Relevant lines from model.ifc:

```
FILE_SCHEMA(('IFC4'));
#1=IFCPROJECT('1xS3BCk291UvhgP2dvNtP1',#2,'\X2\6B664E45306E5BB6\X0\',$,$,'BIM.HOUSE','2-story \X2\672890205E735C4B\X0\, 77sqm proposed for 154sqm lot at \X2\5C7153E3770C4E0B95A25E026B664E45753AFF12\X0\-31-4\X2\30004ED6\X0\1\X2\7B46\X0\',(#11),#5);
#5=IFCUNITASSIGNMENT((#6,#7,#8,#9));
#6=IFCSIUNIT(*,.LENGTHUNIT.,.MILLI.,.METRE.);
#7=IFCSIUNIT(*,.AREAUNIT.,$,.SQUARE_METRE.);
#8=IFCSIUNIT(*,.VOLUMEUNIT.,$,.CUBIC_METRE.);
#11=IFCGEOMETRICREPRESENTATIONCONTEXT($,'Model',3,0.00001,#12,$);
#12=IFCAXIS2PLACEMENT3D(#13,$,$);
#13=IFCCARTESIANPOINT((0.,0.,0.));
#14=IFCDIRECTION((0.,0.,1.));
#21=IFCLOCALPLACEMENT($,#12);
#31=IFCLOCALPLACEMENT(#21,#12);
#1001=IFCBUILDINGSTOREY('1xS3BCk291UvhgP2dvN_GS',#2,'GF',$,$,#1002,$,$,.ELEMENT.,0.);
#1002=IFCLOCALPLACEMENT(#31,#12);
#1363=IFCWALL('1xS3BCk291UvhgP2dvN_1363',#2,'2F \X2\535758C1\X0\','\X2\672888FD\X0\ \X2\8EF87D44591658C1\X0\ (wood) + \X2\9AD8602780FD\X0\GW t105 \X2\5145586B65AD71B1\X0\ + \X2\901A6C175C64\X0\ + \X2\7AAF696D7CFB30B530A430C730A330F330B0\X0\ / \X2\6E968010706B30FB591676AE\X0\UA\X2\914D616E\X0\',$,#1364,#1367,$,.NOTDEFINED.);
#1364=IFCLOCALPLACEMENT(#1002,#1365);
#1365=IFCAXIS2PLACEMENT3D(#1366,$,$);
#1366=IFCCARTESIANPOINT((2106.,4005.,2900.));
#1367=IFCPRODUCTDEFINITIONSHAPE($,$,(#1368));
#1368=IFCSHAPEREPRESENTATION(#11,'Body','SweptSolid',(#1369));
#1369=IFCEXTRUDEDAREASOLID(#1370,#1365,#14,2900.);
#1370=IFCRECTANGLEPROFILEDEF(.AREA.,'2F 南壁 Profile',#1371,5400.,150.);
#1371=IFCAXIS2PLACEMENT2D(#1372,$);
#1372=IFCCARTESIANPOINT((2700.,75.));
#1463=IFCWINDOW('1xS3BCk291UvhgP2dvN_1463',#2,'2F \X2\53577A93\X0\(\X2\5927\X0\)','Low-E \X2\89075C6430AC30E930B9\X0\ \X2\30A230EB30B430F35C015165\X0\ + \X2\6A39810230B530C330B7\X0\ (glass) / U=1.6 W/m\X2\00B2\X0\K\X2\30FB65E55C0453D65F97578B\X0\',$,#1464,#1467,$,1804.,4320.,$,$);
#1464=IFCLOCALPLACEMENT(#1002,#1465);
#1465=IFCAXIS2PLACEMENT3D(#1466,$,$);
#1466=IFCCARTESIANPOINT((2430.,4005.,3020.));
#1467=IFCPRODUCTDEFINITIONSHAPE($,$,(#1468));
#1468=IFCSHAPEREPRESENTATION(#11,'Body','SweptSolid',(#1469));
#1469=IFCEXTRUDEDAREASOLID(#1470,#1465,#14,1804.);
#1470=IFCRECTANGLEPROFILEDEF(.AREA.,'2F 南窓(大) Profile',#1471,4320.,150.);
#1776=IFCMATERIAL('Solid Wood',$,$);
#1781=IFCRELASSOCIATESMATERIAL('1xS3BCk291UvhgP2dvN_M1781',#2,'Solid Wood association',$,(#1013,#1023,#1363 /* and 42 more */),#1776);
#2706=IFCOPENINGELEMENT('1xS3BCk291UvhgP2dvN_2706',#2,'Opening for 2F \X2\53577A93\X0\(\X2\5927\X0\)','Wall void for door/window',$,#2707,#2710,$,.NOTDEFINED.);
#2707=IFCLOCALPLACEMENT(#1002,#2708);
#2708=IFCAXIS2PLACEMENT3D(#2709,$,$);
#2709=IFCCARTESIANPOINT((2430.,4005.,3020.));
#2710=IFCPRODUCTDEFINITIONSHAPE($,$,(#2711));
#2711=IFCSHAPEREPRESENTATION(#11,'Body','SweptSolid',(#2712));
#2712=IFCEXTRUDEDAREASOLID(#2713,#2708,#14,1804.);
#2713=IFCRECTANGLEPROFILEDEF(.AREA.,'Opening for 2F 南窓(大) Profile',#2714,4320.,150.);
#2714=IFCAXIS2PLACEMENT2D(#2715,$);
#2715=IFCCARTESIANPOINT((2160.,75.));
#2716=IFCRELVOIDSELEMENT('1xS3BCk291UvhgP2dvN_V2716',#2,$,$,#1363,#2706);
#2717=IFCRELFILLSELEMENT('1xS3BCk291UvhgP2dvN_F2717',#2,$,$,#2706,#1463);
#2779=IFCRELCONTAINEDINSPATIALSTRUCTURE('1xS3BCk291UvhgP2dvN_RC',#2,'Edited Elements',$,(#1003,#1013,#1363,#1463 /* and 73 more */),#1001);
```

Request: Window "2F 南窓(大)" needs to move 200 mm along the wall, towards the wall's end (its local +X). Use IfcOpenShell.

```python
import ifcopenshell
import ifcopenshell.api.geometry
import ifcopenshell.util.placement

model = ifcopenshell.open("model.ifc")

window = model.by_guid("1xS3BCk291UvhgP2dvN_1463")
opening = window.FillsVoids[0].RelatingOpeningElement
wall = opening.VoidsElements[0].RelatingBuildingElement

wall_matrix = ifcopenshell.util.placement.get_local_placement(wall.ObjectPlacement)
shift = wall_matrix[:3, 0] * 200.0
before = ifcopenshell.util.placement.get_local_placement(window.ObjectPlacement)[:3, 3].copy()

# The window is not placed relative to its opening, so move both.
for product in (opening, window):
    matrix = ifcopenshell.util.placement.get_local_placement(product.ObjectPlacement)
    matrix[:3, 3] += shift
    ifcopenshell.api.geometry.edit_object_placement(model, product=product, matrix=matrix, is_si=False)

after = ifcopenshell.util.placement.get_local_placement(window.ObjectPlacement)[:3, 3]
print("window moved by", (after - before).round(3) + 0.0)

model.write("model-out.ifc")
```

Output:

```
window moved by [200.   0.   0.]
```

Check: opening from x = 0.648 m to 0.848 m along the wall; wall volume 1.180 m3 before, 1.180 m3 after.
